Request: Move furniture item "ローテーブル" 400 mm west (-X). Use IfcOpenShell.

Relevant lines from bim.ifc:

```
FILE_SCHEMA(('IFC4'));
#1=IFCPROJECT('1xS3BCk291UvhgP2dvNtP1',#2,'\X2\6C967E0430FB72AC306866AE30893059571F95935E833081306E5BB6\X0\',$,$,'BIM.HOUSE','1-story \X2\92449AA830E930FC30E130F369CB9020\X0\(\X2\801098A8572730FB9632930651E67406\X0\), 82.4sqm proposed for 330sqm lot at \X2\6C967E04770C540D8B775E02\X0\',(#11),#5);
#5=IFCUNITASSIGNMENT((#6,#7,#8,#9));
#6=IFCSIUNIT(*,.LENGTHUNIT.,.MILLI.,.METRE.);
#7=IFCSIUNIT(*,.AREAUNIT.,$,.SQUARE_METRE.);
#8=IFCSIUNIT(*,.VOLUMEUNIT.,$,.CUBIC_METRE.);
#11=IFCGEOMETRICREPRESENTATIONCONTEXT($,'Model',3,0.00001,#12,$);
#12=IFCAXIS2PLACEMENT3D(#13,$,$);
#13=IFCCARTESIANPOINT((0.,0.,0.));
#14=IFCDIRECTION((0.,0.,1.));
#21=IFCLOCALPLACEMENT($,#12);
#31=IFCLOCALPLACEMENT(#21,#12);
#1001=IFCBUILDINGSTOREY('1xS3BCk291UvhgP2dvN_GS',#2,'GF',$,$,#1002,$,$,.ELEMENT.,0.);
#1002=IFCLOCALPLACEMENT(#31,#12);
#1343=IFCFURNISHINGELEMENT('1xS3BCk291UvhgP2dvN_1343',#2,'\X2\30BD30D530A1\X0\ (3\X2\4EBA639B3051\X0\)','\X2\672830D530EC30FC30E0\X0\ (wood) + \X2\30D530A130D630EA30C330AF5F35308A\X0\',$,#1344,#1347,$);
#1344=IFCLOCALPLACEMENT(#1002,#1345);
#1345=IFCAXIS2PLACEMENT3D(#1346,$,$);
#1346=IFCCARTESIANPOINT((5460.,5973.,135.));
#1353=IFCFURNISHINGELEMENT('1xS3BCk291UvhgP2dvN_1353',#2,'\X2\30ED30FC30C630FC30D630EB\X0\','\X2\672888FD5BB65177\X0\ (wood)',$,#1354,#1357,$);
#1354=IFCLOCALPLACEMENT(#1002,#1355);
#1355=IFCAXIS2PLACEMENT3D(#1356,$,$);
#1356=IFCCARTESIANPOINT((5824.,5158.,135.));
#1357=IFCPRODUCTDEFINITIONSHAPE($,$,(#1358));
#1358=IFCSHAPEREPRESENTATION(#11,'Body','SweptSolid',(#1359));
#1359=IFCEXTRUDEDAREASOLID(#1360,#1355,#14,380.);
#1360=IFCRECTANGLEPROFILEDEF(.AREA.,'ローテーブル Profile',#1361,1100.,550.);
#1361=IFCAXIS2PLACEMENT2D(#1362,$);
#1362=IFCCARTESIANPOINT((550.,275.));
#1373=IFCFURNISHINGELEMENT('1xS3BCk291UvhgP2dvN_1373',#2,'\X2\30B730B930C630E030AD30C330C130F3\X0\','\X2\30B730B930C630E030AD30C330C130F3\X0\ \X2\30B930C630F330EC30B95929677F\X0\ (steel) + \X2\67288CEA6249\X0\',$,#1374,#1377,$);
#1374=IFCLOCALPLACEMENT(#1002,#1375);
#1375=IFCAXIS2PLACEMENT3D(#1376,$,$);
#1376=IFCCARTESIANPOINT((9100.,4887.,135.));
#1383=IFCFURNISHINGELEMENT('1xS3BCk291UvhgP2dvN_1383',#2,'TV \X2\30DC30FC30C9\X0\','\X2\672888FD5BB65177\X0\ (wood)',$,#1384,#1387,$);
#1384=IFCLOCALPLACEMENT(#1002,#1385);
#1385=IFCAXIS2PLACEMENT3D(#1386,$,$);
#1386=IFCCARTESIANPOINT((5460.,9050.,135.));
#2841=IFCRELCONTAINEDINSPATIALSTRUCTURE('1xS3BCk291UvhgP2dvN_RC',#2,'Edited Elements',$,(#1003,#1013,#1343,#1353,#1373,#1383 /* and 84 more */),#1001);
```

```python
import ifcopenshell
import ifcopenshell.api.geometry
import ifcopenshell.util.placement

model = ifcopenshell.open("bim.ifc")

item = model.by_guid("1xS3BCk291UvhgP2dvN_1353")
matrix = ifcopenshell.util.placement.get_local_placement(item.ObjectPlacement)
matrix[0, 3] -= 400.0
ifcopenshell.api.geometry.edit_object_placement(model, product=item, matrix=matrix, is_si=False)

print(ifcopenshell.util.placement.get_local_placement(item.ObjectPlacement).round(3) + 0.0)

model.write("bim_rev.ifc")
```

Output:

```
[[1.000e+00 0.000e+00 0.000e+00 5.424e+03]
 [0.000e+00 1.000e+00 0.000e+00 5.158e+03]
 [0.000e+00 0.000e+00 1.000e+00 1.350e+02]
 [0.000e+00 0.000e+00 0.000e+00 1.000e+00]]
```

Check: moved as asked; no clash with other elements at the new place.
